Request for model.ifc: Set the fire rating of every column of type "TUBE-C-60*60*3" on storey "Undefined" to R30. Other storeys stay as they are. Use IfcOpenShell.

First a look at what the model holds.

```python
import ifcopenshell
import ifcopenshell.util.element

model = ifcopenshell.open("model.ifc")
print(model.schema)
storey = next(s for s in model.by_type("IfcBuildingStorey") if s.Name == "Undefined")
columns = [e for e in ifcopenshell.util.element.get_decomposition(storey) if e.is_a("IfcColumn")]
seen = {}
for e in columns:
    element_type = ifcopenshell.util.element.get_type(e)
    key = (element_type.Name if element_type != e and element_type else None, ifcopenshell.util.element.get_pset(e, "Pset_ColumnCommon", "FireRating"))
    seen[key] = seen.get(key, 0) + 1
for (name, value), count in sorted(seen.items(), key=str):
    print(count, "x", name, "|", value)
```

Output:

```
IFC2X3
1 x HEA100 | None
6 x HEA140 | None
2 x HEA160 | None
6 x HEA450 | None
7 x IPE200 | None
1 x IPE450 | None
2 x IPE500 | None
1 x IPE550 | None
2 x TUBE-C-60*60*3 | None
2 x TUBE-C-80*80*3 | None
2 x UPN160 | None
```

```python
import ifcopenshell
import ifcopenshell.api.pset
import ifcopenshell.util.element

model = ifcopenshell.open("model.ifc")

storey = next(s for s in model.by_type("IfcBuildingStorey") if s.Name == "Undefined")
columns = [e for e in ifcopenshell.util.element.get_decomposition(storey) if e.is_a("IfcColumn")]

count = 0
for e in columns:
    element_type = ifcopenshell.util.element.get_type(e)
    if element_type in (None, e) or element_type.Name != "TUBE-C-60*60*3":
        continue
    # add_pset returns the element's existing set when there is one.
    pset = ifcopenshell.api.pset.add_pset(model, product=e, name="Pset_ColumnCommon")
    ifcopenshell.api.pset.edit_pset(model, pset=pset, properties={"FireRating": "R30"})
    count += 1

print(count, "columns updated")

model.write("model-out.ifc")
```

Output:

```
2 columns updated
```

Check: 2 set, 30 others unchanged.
